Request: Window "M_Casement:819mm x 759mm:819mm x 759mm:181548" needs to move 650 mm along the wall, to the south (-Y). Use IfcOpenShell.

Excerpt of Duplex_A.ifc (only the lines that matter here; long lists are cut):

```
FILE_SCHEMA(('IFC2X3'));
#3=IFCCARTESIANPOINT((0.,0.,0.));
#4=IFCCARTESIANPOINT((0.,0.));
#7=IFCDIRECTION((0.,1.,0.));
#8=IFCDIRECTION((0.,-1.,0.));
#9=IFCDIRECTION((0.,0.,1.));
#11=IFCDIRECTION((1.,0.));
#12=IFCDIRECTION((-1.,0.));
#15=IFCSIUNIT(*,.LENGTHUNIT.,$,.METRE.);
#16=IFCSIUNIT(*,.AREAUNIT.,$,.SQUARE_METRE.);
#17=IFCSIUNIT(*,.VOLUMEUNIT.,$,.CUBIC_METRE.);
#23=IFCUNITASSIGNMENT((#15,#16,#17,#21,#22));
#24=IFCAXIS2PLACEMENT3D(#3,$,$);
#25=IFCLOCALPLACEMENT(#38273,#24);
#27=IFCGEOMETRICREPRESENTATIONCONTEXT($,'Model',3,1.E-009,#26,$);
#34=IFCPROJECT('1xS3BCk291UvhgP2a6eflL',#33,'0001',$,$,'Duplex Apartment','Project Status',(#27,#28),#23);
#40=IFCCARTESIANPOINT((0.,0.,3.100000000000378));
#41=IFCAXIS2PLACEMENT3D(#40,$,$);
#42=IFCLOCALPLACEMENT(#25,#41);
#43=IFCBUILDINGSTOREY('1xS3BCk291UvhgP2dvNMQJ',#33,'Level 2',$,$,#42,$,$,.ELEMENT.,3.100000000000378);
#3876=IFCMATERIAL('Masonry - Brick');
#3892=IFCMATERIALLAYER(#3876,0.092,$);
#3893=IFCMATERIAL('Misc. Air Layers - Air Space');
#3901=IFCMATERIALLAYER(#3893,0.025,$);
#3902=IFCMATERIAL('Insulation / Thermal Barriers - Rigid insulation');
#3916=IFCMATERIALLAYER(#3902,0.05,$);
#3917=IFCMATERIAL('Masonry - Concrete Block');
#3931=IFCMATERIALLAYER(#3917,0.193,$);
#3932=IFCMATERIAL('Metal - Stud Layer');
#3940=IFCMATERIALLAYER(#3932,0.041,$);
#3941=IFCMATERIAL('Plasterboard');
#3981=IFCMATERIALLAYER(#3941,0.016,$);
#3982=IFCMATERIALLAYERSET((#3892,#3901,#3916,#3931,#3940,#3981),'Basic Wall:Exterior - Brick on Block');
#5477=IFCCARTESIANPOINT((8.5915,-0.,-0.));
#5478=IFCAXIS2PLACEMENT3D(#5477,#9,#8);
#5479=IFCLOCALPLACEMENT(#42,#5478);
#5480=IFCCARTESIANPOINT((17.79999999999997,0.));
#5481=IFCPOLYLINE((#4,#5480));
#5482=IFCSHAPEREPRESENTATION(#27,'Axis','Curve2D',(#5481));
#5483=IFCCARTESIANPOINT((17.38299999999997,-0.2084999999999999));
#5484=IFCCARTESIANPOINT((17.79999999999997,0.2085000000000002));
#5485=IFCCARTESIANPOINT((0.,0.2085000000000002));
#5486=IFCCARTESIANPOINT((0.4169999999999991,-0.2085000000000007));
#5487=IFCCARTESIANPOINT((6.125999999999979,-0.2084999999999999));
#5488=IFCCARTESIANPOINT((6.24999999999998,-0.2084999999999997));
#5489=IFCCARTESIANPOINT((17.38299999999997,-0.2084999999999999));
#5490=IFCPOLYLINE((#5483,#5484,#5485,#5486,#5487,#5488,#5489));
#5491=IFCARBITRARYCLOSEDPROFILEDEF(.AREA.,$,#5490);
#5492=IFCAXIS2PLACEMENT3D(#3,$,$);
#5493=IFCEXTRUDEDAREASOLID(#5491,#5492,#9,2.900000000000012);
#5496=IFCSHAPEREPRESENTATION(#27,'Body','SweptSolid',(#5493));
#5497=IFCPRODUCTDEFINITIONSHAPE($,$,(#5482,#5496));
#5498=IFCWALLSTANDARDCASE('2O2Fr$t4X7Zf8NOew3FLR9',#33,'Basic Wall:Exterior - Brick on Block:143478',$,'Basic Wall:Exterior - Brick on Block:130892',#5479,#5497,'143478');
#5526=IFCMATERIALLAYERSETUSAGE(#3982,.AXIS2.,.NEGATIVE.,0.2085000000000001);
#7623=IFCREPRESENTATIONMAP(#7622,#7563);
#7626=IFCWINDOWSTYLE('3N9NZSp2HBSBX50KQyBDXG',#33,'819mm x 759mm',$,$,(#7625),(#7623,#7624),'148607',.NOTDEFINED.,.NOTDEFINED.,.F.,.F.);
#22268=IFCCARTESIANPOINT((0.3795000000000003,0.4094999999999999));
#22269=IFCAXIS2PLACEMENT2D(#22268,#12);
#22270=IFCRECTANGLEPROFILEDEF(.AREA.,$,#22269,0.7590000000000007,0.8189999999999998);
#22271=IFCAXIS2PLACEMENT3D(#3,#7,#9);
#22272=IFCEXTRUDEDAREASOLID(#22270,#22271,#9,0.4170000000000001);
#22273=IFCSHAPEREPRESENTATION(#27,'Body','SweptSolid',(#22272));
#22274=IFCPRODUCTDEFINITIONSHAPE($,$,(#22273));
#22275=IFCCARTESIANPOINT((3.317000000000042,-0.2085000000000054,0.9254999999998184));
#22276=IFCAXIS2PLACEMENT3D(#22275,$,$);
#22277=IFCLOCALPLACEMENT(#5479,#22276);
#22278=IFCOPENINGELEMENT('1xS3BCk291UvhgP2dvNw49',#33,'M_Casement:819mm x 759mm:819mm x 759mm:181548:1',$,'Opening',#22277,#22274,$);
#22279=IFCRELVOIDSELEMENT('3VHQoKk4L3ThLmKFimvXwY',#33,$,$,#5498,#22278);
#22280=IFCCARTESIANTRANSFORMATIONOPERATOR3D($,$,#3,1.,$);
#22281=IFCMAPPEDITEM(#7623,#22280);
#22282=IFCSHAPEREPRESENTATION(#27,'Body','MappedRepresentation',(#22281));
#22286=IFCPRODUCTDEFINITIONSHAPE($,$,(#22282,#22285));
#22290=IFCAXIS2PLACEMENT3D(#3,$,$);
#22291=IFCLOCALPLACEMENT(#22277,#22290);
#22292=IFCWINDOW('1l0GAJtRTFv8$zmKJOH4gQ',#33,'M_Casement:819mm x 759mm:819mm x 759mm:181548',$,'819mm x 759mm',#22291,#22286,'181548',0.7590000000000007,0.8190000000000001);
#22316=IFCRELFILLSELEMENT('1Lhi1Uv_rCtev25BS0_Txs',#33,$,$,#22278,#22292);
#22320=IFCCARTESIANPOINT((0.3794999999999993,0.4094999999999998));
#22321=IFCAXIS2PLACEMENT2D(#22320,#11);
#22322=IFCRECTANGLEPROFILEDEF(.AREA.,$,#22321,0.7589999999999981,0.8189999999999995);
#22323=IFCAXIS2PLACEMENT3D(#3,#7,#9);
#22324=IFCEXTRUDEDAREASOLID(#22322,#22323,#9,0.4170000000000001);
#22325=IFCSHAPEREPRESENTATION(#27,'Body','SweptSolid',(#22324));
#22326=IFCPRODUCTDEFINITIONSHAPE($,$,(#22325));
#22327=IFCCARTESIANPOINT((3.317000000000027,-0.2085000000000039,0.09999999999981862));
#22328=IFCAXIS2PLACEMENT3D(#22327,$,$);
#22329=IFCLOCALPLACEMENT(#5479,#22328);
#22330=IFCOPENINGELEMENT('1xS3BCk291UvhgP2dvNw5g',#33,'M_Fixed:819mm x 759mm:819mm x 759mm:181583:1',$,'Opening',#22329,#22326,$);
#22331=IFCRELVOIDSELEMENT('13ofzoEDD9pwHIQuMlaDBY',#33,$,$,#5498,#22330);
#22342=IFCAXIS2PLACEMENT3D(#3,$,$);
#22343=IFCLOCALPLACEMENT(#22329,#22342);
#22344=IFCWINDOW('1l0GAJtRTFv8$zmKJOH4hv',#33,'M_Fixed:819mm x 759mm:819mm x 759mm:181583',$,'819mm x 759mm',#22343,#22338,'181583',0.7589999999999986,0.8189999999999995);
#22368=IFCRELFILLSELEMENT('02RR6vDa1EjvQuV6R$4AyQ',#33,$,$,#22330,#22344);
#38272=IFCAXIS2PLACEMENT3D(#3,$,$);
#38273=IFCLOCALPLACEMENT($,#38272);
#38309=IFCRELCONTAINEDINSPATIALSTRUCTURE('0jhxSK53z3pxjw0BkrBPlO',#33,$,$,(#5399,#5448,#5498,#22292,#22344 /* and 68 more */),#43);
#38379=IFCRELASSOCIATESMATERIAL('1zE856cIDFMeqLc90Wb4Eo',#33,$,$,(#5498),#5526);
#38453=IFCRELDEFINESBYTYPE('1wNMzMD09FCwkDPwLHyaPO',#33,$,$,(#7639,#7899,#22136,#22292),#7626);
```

```python
import ifcopenshell
import ifcopenshell.api.geometry
import ifcopenshell.util.placement

model = ifcopenshell.open("Duplex_A.ifc")

window = model.by_guid("1l0GAJtRTFv8$zmKJOH4gQ")
opening = window.FillsVoids[0].RelatingOpeningElement
wall = opening.VoidsElements[0].RelatingBuildingElement

wall_matrix = ifcopenshell.util.placement.get_local_placement(wall.ObjectPlacement)
shift = wall_matrix[:3, 0] * 0.65
before = ifcopenshell.util.placement.get_local_placement(window.ObjectPlacement)[:3, 3].copy()

# The window is placed relative to its opening, so it follows when the opening moves.
matrix = ifcopenshell.util.placement.get_local_placement(opening.ObjectPlacement)
matrix[:3, 3] += shift
ifcopenshell.api.geometry.edit_object_placement(
    model, product=opening, matrix=matrix, is_si=False, should_transform_children=True
)

after = ifcopenshell.util.placement.get_local_placement(window.ObjectPlacement)[:3, 3]
print("window moved by", (after - before).round(3) + 0.0)

model.write("Duplex_A_rev.ifc")
```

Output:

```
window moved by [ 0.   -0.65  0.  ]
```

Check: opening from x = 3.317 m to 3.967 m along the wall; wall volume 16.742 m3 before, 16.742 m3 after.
